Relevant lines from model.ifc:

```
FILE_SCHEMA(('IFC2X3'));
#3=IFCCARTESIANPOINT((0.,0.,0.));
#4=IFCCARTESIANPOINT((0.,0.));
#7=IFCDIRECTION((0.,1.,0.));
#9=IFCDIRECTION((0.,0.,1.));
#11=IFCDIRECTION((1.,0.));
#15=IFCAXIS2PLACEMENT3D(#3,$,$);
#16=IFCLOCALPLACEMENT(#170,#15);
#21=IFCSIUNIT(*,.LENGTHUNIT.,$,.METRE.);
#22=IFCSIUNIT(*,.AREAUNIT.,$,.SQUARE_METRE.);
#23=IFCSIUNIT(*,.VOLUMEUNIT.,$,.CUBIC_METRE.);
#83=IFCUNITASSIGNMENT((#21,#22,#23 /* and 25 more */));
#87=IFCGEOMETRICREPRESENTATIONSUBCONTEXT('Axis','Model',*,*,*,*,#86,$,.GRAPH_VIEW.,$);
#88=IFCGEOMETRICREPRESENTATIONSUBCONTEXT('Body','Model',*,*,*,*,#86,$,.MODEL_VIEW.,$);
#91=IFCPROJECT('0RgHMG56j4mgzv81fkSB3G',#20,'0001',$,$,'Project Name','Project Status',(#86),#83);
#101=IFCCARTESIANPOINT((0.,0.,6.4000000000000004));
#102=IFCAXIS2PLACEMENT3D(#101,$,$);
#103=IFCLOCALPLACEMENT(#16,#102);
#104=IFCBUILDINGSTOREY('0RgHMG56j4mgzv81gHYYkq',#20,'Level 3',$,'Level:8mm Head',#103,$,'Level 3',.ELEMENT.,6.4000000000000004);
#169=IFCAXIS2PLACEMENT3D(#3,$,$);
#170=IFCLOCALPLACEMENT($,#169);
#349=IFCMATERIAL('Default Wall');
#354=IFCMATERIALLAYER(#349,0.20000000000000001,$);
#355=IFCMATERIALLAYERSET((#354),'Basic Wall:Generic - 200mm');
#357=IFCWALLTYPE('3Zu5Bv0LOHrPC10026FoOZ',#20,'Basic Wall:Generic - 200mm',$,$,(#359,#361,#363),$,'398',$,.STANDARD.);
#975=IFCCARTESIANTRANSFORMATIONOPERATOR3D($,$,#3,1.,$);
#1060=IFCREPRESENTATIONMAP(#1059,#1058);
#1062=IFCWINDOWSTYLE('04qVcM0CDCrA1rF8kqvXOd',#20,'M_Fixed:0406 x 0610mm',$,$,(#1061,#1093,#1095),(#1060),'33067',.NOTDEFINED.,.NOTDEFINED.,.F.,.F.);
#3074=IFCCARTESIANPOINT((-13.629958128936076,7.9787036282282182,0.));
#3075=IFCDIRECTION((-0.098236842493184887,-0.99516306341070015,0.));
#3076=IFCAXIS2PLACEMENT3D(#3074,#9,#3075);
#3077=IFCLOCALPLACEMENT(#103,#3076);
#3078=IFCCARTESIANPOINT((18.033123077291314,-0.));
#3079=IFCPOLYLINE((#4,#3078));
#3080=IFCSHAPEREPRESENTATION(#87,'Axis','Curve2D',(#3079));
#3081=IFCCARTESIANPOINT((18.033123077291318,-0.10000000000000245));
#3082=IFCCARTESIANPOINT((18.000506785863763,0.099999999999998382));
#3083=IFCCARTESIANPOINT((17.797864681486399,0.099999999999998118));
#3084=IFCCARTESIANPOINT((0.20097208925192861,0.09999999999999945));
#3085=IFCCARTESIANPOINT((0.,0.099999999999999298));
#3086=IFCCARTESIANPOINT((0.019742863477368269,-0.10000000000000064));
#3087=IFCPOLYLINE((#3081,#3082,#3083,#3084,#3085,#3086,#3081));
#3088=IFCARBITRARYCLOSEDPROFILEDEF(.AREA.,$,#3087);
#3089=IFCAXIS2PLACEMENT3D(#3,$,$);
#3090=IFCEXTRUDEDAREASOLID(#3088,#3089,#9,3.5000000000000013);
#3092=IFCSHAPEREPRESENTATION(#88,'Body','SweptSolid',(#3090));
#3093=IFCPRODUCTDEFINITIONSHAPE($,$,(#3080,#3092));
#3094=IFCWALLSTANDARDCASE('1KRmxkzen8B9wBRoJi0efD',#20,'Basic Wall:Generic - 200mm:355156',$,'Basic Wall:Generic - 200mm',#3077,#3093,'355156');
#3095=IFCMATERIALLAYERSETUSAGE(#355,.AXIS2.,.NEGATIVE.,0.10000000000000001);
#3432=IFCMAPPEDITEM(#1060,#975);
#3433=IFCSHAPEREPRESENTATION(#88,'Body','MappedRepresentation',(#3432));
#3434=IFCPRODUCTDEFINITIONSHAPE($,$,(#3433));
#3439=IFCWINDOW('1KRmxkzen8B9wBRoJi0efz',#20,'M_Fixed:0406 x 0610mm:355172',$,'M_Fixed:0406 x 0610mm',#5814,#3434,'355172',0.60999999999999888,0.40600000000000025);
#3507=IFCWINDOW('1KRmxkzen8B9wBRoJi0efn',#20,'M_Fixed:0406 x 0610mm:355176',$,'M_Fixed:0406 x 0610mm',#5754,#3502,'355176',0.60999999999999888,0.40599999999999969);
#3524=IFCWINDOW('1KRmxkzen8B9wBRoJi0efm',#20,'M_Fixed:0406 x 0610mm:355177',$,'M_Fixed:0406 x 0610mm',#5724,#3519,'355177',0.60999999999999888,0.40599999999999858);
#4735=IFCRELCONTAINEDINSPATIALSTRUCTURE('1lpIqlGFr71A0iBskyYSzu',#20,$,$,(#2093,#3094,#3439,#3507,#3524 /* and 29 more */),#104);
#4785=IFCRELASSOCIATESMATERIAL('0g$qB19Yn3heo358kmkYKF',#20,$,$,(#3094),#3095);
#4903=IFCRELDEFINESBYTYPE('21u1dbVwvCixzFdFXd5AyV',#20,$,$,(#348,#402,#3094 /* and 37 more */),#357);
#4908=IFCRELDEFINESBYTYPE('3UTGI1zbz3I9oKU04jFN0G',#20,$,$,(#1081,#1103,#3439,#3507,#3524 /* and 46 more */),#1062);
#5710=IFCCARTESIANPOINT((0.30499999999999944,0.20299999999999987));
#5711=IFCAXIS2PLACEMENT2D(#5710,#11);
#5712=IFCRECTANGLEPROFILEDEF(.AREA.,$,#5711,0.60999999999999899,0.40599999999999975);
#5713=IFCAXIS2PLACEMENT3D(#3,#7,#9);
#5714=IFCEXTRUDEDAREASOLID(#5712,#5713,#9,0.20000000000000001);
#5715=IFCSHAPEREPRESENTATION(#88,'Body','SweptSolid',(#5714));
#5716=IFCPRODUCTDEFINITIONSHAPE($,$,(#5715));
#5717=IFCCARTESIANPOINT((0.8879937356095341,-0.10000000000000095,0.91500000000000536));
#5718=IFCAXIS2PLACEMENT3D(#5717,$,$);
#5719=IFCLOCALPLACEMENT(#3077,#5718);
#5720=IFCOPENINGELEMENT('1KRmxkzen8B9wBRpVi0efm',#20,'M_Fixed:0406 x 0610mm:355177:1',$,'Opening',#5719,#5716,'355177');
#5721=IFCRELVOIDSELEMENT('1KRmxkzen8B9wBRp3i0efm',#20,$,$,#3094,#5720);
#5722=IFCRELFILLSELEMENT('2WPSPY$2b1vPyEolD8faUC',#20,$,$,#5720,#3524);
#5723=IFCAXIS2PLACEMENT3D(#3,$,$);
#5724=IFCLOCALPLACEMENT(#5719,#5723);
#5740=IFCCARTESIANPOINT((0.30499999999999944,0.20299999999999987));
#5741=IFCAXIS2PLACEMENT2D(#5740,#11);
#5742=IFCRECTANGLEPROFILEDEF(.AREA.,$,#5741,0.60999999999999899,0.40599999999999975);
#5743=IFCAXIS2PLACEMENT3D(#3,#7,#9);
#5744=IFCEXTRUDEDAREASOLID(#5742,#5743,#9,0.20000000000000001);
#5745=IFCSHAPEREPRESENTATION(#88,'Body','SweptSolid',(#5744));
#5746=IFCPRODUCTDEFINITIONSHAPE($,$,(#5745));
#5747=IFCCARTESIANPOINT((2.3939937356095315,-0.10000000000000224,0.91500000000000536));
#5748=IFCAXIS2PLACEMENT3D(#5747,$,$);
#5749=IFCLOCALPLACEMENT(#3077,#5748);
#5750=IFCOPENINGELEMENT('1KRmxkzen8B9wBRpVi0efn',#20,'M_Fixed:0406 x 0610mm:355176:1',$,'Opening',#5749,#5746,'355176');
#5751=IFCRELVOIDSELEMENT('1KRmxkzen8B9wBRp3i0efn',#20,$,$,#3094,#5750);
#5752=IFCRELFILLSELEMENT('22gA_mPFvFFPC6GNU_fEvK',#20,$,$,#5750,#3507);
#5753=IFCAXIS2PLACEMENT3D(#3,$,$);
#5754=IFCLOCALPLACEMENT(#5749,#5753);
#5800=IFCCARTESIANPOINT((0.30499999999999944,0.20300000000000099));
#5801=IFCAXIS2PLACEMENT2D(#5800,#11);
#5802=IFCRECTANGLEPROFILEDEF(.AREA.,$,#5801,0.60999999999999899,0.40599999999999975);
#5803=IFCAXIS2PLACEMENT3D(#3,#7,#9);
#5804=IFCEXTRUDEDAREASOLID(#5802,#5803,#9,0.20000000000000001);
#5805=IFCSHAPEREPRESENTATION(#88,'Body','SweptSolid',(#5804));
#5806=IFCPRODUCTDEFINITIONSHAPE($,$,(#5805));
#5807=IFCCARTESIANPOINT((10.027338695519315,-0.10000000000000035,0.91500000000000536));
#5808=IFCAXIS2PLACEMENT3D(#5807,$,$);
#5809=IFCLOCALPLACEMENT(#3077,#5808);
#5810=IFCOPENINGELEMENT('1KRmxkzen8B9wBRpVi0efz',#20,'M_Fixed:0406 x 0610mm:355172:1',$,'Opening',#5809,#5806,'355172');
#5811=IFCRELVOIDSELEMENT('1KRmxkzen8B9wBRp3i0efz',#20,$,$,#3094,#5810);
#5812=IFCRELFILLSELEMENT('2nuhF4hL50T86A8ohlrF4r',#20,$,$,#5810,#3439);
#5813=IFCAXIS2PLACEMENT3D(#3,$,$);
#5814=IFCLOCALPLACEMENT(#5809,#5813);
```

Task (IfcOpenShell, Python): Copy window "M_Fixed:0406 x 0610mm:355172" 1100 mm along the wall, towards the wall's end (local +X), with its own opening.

```python
import ifcopenshell
import ifcopenshell.api.feature
import ifcopenshell.api.geometry
import ifcopenshell.api.root
import ifcopenshell.geom
import ifcopenshell.util.element
import ifcopenshell.util.placement
import ifcopenshell.util.shape
import ifcopenshell.util.unit

model = ifcopenshell.open("model.ifc")
unit_scale = ifcopenshell.util.unit.calculate_unit_scale(model)
settings = ifcopenshell.geom.settings()


def volume(element):
    """Net volume in cubic metres, openings subtracted."""
    shape = ifcopenshell.geom.create_shape(settings, element)
    return ifcopenshell.util.shape.get_volume(shape.geometry)


def reuse_history(source, copy):
    """copy_class also copies each property set's owner history, people and application; keep the originals."""
    for rel in copy.IsDefinedBy:
        if rel.is_a("IfcRelDefinesByProperties") and (history := rel.RelatingPropertyDefinition.OwnerHistory):
            rel.RelatingPropertyDefinition.OwnerHistory = source.OwnerHistory
            ifcopenshell.util.element.remove_deep2(model, history)


window = model.by_guid("1KRmxkzen8B9wBRoJi0efz")
opening = window.FillsVoids[0].RelatingOpeningElement
wall = opening.VoidsElements[0].RelatingBuildingElement
before = volume(wall)
shift = ifcopenshell.util.placement.get_local_placement(wall.ObjectPlacement)[:3, 0] * 1.1 / unit_scale

# copy_class copies the void relationship, type, container and properties, but no geometry.
new_opening = ifcopenshell.api.root.copy_class(model, product=opening)
new_opening.Representation = ifcopenshell.util.element.copy_deep(
    model, opening.Representation, exclude=["IfcGeometricRepresentationContext", "IfcRepresentationMap"]
)
new_opening.Name = "M_Fixed:0406 x 0610mm"
new_opening.Tag = None
new_window = ifcopenshell.api.root.copy_class(model, product=window)
new_window.Representation = ifcopenshell.util.element.copy_deep(
    model, window.Representation, exclude=["IfcGeometricRepresentationContext", "IfcRepresentationMap"]
)
new_window.Name = "M_Fixed:0406 x 0610mm"
new_window.Tag = None
reuse_history(window, new_window)
fills = ifcopenshell.api.feature.add_filling(model, opening=new_opening, element=new_window)
fills.OwnerHistory = new_window.OwnerHistory  # required in IFC2X3

for old, new in ((opening, new_opening), (window, new_window)):
    matrix = ifcopenshell.util.placement.get_local_placement(old.ObjectPlacement)
    matrix[:3, 3] += shift
    ifcopenshell.api.geometry.edit_object_placement(model, product=new, matrix=matrix, is_si=False)

after = volume(wall)

print(f"wall volume {before:.3f} -> {after:.3f} m3")

model.write("model_updated.ifc")
```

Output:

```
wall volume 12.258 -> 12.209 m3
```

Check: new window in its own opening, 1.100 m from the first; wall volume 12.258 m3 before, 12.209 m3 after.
